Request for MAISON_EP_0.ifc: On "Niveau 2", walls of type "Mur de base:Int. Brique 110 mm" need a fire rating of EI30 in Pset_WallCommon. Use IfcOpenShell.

First a look at what the model holds.

```python
import ifcopenshell
import ifcopenshell.util.element

model = ifcopenshell.open("MAISON_EP_0.ifc")
print(model.schema)
storey = next(s for s in model.by_type("IfcBuildingStorey") if s.Name == "Niveau 2")
walls = [e for e in ifcopenshell.util.element.get_decomposition(storey) if e.is_a("IfcWall")]
seen = {}
for e in walls:
    element_type = ifcopenshell.util.element.get_type(e)
    key = (element_type.Name if element_type != e and element_type else None, ifcopenshell.util.element.get_pset(e, "Pset_WallCommon", "FireRating"))
    seen[key] = seen.get(key, 0) + 1
for (name, value), count in sorted(seen.items(), key=str):
    print(count, "x", name, "|", value)
```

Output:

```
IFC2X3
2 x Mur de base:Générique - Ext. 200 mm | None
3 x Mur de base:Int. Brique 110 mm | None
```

```python
import ifcopenshell
import ifcopenshell.api.pset
import ifcopenshell.util.element

model = ifcopenshell.open("MAISON_EP_0.ifc")

storey = next(s for s in model.by_type("IfcBuildingStorey") if s.Name == "Niveau 2")
walls = [e for e in ifcopenshell.util.element.get_decomposition(storey) if e.is_a("IfcWall")]

count = 0
for e in walls:
    element_type = ifcopenshell.util.element.get_type(e)
    if element_type in (None, e) or element_type.Name != "Mur de base:Int. Brique 110 mm":
        continue
    found = ifcopenshell.util.element.get_pset(e, "Pset_WallCommon", should_inherit=False)
    if found:
        pset = model.by_id(found["id"])
        if len(ifcopenshell.util.element.get_elements_by_pset(pset)) > 1:
            pset = ifcopenshell.api.pset.unshare_pset(model, products=[e], pset=pset)[0]
    else:
        pset = ifcopenshell.api.pset.add_pset(model, product=e, name="Pset_WallCommon")
    ifcopenshell.api.pset.edit_pset(model, pset=pset, properties={"FireRating": "EI30"})
    count += 1

print(count, "walls updated")

model.write("MAISON_EP_0-out.ifc")
```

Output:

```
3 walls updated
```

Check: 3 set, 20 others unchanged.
